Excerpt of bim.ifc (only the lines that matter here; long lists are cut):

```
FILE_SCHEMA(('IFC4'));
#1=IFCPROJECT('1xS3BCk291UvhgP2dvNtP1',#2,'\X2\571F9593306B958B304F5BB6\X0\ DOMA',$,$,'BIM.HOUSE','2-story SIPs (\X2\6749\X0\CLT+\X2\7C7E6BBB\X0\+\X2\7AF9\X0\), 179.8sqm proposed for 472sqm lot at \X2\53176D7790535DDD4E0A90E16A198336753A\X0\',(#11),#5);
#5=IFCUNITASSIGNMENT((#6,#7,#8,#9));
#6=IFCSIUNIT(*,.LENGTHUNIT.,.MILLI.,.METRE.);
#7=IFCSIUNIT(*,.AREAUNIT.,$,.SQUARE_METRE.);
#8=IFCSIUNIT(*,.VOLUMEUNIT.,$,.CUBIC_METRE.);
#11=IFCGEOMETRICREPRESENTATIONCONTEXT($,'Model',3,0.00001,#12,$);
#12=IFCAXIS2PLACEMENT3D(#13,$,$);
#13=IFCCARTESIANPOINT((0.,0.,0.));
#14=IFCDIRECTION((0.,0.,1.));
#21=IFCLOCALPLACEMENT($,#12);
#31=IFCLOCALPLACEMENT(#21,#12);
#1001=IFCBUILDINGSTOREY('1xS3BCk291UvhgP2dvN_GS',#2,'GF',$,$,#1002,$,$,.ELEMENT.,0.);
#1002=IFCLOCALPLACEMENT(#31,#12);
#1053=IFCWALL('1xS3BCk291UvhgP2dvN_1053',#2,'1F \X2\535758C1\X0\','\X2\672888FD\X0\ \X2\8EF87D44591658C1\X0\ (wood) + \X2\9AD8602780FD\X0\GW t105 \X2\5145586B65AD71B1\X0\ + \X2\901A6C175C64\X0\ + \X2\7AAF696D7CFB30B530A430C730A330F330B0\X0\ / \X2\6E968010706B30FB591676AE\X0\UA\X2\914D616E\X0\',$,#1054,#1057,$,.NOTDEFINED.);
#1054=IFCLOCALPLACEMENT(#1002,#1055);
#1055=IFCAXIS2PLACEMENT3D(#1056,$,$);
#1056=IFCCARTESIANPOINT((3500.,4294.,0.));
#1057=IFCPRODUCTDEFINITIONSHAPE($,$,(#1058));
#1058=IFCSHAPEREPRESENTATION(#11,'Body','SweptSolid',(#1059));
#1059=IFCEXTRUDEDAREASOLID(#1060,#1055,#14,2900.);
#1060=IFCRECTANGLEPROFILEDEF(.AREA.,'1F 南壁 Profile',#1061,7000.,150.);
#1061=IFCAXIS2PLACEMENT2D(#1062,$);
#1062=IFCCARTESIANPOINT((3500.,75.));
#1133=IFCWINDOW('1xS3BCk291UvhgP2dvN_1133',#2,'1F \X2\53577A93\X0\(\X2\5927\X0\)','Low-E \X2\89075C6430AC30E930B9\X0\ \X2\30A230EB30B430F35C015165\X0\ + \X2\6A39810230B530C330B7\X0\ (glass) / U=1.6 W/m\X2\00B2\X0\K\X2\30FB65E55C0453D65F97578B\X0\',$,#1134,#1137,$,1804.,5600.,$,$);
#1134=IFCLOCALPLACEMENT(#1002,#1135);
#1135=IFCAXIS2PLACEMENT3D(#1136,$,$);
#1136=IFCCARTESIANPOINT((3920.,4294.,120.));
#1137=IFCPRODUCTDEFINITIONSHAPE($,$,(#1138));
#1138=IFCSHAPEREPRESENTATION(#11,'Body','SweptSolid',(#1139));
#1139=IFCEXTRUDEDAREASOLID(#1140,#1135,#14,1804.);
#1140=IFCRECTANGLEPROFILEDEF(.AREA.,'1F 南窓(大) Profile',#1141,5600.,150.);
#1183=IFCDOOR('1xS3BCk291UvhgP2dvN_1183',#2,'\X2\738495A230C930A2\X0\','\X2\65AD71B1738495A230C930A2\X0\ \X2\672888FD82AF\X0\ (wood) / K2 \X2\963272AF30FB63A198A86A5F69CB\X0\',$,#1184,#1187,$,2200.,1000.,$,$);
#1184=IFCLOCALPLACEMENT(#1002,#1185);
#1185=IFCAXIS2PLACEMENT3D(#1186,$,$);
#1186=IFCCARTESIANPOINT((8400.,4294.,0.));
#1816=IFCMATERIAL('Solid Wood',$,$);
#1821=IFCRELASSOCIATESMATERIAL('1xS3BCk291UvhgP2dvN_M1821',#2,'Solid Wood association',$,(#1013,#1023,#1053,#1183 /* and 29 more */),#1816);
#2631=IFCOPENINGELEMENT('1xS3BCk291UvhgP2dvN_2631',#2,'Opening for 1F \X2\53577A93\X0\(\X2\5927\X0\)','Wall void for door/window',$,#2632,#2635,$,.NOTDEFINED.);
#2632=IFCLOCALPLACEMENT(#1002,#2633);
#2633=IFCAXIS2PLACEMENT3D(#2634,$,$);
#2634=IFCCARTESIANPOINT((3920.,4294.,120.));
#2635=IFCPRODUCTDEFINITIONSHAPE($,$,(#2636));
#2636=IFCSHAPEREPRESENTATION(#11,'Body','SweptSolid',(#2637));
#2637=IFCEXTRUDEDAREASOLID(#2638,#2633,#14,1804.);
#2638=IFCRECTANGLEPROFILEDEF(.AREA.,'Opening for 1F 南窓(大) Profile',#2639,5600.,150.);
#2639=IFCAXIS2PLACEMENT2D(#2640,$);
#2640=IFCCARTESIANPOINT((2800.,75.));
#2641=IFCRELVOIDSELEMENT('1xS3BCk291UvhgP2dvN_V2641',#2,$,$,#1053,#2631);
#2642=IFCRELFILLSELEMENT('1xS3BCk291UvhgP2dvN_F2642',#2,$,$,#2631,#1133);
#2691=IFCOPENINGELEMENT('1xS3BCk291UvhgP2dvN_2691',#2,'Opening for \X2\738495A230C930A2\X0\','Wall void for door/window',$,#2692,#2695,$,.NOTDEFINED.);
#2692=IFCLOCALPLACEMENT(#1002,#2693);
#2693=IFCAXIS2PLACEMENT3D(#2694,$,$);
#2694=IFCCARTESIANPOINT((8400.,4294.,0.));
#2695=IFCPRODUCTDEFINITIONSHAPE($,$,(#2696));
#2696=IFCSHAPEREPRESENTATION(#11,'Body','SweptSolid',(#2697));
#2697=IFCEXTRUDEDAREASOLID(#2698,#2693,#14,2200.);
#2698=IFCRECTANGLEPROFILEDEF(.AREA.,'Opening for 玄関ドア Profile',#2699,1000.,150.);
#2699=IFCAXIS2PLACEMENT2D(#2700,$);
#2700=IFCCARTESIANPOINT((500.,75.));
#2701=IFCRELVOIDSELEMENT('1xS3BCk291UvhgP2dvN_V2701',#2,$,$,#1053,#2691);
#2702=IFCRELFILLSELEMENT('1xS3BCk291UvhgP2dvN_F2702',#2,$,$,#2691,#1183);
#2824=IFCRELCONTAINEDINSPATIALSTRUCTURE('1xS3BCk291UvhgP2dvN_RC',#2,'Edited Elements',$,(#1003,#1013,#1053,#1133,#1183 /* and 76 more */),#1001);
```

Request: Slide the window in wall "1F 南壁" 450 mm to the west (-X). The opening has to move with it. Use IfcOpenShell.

```python
import ifcopenshell
import ifcopenshell.api.geometry
import ifcopenshell.util.placement
import ifcopenshell.util.unit

model = ifcopenshell.open("bim.ifc")
unit_scale = ifcopenshell.util.unit.calculate_unit_scale(model)

window = model.by_guid("1xS3BCk291UvhgP2dvN_1133")
opening = window.FillsVoids[0].RelatingOpeningElement
wall = opening.VoidsElements[0].RelatingBuildingElement

wall_matrix = ifcopenshell.util.placement.get_local_placement(wall.ObjectPlacement)
shift = wall_matrix[:3, 0] * -0.45 / unit_scale
before = ifcopenshell.util.placement.get_local_placement(window.ObjectPlacement)[:3, 3].copy()

# The window is not placed relative to its opening, so move both.
for product in (opening, window):
    matrix = ifcopenshell.util.placement.get_local_placement(product.ObjectPlacement)
    matrix[:3, 3] += shift
    ifcopenshell.api.geometry.edit_object_placement(model, product=product, matrix=matrix, is_si=False)

after = ifcopenshell.util.placement.get_local_placement(window.ObjectPlacement)[:3, 3]
print("window moved by", (after - before).round(3) + 0.0)

model.write("bim_rev.ifc")
```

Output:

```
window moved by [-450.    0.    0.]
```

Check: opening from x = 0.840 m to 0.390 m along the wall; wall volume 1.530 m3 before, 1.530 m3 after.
